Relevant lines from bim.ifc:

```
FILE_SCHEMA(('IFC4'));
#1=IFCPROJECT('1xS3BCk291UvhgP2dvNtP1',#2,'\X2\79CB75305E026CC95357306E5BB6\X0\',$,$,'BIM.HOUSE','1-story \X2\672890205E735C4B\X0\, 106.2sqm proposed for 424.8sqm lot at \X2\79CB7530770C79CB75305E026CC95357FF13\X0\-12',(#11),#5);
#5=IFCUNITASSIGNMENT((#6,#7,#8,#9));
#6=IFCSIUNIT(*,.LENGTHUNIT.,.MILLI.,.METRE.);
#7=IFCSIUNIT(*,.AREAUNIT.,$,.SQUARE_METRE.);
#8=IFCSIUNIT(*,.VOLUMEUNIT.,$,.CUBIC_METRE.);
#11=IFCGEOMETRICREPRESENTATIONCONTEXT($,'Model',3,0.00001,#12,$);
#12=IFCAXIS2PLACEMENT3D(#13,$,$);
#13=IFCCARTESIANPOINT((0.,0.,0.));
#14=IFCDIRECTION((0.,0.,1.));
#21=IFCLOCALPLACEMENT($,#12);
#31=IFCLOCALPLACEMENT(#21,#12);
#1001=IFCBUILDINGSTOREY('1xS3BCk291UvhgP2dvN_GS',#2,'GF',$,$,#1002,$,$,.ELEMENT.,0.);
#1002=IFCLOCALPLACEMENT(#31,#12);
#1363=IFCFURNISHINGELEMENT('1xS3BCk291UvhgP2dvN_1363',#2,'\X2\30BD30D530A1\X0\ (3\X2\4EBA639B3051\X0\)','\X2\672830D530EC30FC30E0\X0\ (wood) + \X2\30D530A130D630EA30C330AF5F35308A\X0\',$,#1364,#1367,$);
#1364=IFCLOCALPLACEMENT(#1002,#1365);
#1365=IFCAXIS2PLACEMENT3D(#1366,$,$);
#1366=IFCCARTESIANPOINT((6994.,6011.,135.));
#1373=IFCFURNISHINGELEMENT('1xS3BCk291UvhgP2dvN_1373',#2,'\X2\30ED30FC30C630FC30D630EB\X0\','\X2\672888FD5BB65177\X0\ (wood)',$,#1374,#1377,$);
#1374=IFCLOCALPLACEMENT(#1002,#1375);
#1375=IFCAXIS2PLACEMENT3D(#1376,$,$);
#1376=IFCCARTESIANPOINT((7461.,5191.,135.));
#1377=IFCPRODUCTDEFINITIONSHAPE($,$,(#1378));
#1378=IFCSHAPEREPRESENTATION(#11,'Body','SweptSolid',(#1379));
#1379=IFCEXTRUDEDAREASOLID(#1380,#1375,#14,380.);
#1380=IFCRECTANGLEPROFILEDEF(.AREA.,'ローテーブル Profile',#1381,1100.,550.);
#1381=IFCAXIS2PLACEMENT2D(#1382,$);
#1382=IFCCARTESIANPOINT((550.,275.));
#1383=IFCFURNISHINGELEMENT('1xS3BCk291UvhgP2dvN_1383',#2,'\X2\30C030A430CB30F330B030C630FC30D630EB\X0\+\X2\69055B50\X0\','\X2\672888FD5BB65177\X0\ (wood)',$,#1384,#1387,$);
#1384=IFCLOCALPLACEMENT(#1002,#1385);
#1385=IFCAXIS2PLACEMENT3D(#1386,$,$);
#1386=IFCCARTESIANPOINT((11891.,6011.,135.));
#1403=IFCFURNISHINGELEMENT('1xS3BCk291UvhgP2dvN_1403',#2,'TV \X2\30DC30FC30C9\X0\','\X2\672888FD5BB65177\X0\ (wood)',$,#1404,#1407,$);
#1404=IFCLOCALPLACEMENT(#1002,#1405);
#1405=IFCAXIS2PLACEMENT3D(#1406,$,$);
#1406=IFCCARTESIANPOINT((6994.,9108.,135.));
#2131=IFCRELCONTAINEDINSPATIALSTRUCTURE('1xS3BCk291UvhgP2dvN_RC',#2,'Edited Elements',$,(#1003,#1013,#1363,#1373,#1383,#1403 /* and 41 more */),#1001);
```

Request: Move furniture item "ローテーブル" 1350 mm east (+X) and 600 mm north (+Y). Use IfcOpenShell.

```python
import ifcopenshell
import ifcopenshell.api.geometry
import ifcopenshell.util.placement
import ifcopenshell.util.unit

model = ifcopenshell.open("bim.ifc")
unit_scale = ifcopenshell.util.unit.calculate_unit_scale(model)

item = model.by_id(1373)
matrix = ifcopenshell.util.placement.get_local_placement(item.ObjectPlacement)
matrix[0, 3] += 1.35 / unit_scale
matrix[1, 3] += 0.6 / unit_scale
ifcopenshell.api.geometry.edit_object_placement(model, product=item, matrix=matrix, is_si=False)

print(ifcopenshell.util.placement.get_local_placement(item.ObjectPlacement).round(3) + 0.0)

model.write("bim_v2.ifc")
```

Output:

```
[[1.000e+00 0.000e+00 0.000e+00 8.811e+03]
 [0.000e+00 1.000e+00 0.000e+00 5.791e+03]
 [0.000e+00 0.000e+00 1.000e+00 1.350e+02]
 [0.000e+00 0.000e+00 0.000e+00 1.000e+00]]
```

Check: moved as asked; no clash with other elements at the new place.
